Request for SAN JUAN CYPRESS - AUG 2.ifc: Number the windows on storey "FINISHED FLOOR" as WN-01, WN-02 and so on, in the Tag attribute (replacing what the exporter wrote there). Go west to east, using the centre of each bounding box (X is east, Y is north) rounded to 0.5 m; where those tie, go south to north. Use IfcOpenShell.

First a look at what the model holds.

```python
import ifcopenshell
import ifcopenshell.util.element
import ifcopenshell.util.placement

model = ifcopenshell.open("SAN JUAN CYPRESS - AUG 2.ifc")
print(model.schema)
storey = next(s for s in model.by_type("IfcBuildingStorey") if s.Name == "FINISHED FLOOR")
windows = [e for e in ifcopenshell.util.element.get_decomposition(storey) if e.is_a("IfcWindow")]
for e in sorted(windows, key=lambda e: e.id()):
    origin = ifcopenshell.util.placement.get_local_placement(e.ObjectPlacement)[:3, 3]
    print(e.id(), e.Tag, e.Name, origin.round(2) + 0.0, sep=" | ")
```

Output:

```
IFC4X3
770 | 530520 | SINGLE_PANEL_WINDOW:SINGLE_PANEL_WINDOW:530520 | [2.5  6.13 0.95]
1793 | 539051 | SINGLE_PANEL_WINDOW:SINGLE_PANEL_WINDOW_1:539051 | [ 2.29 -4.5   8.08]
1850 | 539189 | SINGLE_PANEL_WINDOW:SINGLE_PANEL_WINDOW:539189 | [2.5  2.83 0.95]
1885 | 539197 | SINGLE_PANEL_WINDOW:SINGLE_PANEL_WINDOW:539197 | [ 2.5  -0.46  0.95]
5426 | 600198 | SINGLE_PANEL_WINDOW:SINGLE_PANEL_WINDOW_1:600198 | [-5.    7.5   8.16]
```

```python
import ifcopenshell
import ifcopenshell.geom
import ifcopenshell.util.element
import ifcopenshell.util.shape

model = ifcopenshell.open("SAN JUAN CYPRESS - AUG 2.ifc")
settings = ifcopenshell.geom.settings()
settings.set("use-world-coords", True)


def centre(element):
    shape = ifcopenshell.geom.create_shape(settings, element)
    return ifcopenshell.util.shape.get_bbox_centroid(shape.geometry)


storey = next(s for s in model.by_type("IfcBuildingStorey") if s.Name == "FINISHED FLOOR")
windows = [e for e in ifcopenshell.util.element.get_decomposition(storey) if e.is_a("IfcWindow")]

# Insertion points can sit at a corner or the storey origin, so sort by the geometry (in metres).
centres = {e: centre(e) for e in windows}
windows.sort(key=lambda e: (round(centres[e][0] / 0.5), centres[e][1]))

for i, e in enumerate(windows, start=1):
    number = f"WN-{i:02d}"
    e.Tag = number
    print(e.id(), number)

model.write("SAN JUAN CYPRESS - AUG 2-out.ifc")
```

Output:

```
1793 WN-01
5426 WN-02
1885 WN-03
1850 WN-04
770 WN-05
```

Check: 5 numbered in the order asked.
